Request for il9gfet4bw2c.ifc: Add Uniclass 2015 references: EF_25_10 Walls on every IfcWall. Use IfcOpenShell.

First a look at what the model holds.

```python
import ifcopenshell

model = ifcopenshell.open("il9gfet4bw2c.ifc")
print(model.schema)
print("classifications:", [c.Name for c in model.by_type("IfcClassification")])
for ifc_class in ("IfcDoor", "IfcRoof", "IfcStair", "IfcWall", "IfcWindow"):
    print(ifc_class, len(model.by_type(ifc_class)))
```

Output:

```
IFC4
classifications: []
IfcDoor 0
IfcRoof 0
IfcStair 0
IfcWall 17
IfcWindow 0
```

```python
import ifcopenshell
import ifcopenshell.api.classification

model = ifcopenshell.open("il9gfet4bw2c.ifc")

system = ifcopenshell.api.classification.add_classification(model, classification="Uniclass 2015")

codes = {
    "IfcWall": ("EF_25_10", "Walls"),
}
for ifc_class, (code, name) in codes.items():
    products = model.by_type(ifc_class)
    ifcopenshell.api.classification.add_reference(
        model, products=products, classification=system, identification=code, name=name
    )
    print(code, len(products))

model.write("il9gfet4bw2c-out.ifc")
```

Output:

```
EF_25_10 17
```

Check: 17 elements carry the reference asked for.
